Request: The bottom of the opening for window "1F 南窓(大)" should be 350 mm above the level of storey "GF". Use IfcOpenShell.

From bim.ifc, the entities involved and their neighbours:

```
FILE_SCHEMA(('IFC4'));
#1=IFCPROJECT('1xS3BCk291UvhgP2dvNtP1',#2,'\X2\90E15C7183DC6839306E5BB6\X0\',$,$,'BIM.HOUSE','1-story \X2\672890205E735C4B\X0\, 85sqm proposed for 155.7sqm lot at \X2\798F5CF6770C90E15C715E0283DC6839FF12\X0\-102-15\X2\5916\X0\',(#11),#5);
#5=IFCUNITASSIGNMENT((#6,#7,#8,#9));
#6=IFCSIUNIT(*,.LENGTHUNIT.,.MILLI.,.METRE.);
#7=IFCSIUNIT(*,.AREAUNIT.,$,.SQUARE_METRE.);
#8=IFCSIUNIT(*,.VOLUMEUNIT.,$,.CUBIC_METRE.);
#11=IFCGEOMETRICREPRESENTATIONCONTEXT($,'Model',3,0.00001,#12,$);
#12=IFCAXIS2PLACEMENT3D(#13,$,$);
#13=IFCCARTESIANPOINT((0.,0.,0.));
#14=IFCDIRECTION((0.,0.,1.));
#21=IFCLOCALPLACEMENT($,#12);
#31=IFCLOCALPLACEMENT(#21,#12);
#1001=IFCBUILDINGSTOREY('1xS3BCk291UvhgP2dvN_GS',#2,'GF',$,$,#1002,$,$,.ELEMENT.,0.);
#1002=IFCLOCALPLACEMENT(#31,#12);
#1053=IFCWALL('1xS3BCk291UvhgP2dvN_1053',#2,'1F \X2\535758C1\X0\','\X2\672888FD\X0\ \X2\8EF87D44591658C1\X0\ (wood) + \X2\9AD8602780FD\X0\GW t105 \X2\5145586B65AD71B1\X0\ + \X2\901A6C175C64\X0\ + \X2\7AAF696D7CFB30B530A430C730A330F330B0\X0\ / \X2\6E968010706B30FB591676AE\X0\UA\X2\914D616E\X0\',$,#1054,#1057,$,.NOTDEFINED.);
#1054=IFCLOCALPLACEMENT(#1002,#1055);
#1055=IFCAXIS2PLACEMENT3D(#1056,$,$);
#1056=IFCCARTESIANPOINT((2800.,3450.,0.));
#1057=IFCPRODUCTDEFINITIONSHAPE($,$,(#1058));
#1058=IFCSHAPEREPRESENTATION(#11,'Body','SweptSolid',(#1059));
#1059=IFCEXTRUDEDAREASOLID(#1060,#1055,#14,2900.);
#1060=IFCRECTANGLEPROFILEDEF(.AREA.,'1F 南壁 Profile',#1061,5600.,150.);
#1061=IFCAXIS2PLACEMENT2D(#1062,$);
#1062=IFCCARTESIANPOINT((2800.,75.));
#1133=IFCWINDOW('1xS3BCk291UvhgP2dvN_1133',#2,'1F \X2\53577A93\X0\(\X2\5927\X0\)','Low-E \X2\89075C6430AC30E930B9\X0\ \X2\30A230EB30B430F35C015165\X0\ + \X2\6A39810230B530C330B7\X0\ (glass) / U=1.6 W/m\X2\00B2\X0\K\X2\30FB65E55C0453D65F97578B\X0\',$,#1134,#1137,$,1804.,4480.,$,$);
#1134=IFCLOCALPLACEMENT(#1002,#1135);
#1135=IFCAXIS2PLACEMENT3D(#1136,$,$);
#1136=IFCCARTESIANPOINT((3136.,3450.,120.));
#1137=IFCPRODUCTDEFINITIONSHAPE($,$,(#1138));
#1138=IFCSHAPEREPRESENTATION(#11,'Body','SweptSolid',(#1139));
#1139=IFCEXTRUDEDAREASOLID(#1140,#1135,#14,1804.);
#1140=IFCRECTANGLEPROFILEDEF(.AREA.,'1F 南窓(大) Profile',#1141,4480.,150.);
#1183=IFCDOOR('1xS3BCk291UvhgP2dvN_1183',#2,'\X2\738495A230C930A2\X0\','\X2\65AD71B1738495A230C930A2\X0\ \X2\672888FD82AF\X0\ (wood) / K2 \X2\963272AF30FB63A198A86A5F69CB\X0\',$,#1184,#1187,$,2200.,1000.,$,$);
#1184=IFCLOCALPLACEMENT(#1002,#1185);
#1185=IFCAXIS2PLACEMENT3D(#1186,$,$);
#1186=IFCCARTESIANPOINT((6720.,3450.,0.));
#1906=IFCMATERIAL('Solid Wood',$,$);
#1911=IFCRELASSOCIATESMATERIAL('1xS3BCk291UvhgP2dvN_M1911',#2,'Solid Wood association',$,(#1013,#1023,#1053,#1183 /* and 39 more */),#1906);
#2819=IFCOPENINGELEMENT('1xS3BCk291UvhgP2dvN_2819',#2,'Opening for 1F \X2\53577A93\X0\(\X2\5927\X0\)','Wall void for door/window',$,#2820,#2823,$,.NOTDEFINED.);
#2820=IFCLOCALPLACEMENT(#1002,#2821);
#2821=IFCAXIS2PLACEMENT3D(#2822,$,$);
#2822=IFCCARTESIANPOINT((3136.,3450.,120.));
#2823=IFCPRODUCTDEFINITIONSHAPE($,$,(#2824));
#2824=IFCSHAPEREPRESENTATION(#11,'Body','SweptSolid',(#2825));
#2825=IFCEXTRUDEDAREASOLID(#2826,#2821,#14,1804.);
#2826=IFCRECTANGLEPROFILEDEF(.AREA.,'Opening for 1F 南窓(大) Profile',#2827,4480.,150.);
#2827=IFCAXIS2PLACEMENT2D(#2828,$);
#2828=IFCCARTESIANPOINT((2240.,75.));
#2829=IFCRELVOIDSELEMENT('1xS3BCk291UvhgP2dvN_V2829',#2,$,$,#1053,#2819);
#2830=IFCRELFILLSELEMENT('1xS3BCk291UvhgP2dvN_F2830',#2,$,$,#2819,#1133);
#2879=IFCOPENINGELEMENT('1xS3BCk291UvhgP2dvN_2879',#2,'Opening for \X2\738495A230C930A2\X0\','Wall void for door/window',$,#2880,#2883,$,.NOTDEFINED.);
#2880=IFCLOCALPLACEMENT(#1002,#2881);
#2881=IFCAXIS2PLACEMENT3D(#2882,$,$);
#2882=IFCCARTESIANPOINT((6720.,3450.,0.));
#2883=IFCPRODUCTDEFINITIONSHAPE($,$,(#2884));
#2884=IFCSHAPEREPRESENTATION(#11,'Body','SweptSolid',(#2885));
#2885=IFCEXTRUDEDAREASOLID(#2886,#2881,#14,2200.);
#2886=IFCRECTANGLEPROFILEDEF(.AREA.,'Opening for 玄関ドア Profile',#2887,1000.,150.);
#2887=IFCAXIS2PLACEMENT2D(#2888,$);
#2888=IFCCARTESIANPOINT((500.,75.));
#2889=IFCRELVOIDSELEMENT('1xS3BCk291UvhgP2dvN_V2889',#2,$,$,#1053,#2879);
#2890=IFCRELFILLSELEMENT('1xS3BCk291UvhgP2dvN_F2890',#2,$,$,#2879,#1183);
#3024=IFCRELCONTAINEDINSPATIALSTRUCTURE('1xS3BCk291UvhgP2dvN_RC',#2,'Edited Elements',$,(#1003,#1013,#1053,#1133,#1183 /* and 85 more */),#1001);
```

```python
import numpy as np
import ifcopenshell
import ifcopenshell.api.geometry
import ifcopenshell.geom
import ifcopenshell.util.element
import ifcopenshell.util.placement
import ifcopenshell.util.shape
import ifcopenshell.util.unit

model = ifcopenshell.open("bim.ifc")
unit_scale = ifcopenshell.util.unit.calculate_unit_scale(model)

window = model.by_guid("1xS3BCk291UvhgP2dvN_1133")
opening = window.FillsVoids[0].RelatingOpeningElement
storey = ifcopenshell.util.element.get_container(window, ifc_class="IfcBuildingStorey")
level = ifcopenshell.util.placement.get_local_placement(storey.ObjectPlacement)[2, 3]

# The opening's origin need not be at the sill, so measure its lowest point.
shape = ifcopenshell.geom.create_shape(ifcopenshell.geom.settings(), opening)
bottom = ifcopenshell.util.shape.get_shape_bottom_elevation(shape, shape.geometry) / unit_scale
dz = level + 0.35 / unit_scale - bottom

shift = np.array([0.0, 0.0, dz])
# The window is not placed relative to its opening, so move both.
for product in (opening, window):
    matrix = ifcopenshell.util.placement.get_local_placement(product.ObjectPlacement)
    matrix[:3, 3] += shift
    ifcopenshell.api.geometry.edit_object_placement(model, product=product, matrix=matrix, is_si=False)

print(f"moved by {dz * unit_scale:+.3f} m")

model.write("bim-out.ifc")
```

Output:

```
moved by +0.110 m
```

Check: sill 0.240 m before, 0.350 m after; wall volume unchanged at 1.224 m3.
